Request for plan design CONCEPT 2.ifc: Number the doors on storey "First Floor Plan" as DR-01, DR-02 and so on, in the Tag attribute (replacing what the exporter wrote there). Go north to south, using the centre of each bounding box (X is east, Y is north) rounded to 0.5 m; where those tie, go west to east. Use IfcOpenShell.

First a look at what the model holds.

```python
import ifcopenshell
import ifcopenshell.util.element
import ifcopenshell.util.placement

model = ifcopenshell.open("plan design CONCEPT 2.ifc")
print(model.schema)
storey = next(s for s in model.by_type("IfcBuildingStorey") if s.Name == "First Floor Plan")
doors = [e for e in ifcopenshell.util.element.get_decomposition(storey) if e.is_a("IfcDoor")]
for e in sorted(doors, key=lambda e: e.id()):
    origin = ifcopenshell.util.placement.get_local_placement(e.ObjectPlacement)[:3, 3]
    print(e.id(), e.Tag, e.Name, origin.round(2) + 0.0, sep=" | ")
```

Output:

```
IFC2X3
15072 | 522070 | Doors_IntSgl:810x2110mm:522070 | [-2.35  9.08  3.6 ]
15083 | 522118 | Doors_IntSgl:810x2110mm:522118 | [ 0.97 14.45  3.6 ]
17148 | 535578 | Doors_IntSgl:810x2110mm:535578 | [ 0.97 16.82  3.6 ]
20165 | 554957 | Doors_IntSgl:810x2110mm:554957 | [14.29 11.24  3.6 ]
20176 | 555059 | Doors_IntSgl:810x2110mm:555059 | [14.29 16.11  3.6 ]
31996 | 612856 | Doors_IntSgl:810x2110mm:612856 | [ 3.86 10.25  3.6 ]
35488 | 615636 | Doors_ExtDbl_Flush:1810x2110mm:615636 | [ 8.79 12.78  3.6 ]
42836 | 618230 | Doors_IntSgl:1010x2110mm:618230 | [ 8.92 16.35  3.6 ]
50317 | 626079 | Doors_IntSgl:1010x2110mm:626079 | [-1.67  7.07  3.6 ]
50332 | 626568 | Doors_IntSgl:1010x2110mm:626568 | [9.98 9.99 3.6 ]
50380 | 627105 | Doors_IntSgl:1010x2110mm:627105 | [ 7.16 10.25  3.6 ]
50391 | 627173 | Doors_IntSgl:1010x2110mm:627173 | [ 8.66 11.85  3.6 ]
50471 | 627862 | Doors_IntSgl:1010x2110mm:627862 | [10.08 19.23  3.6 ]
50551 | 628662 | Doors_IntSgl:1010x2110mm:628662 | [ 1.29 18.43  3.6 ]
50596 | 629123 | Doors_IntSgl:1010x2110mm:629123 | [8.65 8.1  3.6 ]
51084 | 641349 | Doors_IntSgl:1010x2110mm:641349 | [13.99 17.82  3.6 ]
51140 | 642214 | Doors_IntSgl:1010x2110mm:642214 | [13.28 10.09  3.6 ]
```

```python
import ifcopenshell
import ifcopenshell.geom
import ifcopenshell.util.element
import ifcopenshell.util.shape

model = ifcopenshell.open("plan design CONCEPT 2.ifc")
settings = ifcopenshell.geom.settings()
settings.set("use-world-coords", True)


def centre(element):
    shape = ifcopenshell.geom.create_shape(settings, element)
    return ifcopenshell.util.shape.get_bbox_centroid(shape.geometry)


storey = next(s for s in model.by_type("IfcBuildingStorey") if s.Name == "First Floor Plan")
doors = [e for e in ifcopenshell.util.element.get_decomposition(storey) if e.is_a("IfcDoor")]

# Insertion points can sit at a corner or the storey origin, so sort by the geometry (in metres).
centres = {e: centre(e) for e in doors}
doors.sort(key=lambda e: (-round(centres[e][1] / 0.5), centres[e][0]))

for i, e in enumerate(doors, start=1):
    number = f"DR-{i:02d}"
    e.Tag = number
    print(e.id(), number)

model.write("plan design CONCEPT 2_updated.ifc")
```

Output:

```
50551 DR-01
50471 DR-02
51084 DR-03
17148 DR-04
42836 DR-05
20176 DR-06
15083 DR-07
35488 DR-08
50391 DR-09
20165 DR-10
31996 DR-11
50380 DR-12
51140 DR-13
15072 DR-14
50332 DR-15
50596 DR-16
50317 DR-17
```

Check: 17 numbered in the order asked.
